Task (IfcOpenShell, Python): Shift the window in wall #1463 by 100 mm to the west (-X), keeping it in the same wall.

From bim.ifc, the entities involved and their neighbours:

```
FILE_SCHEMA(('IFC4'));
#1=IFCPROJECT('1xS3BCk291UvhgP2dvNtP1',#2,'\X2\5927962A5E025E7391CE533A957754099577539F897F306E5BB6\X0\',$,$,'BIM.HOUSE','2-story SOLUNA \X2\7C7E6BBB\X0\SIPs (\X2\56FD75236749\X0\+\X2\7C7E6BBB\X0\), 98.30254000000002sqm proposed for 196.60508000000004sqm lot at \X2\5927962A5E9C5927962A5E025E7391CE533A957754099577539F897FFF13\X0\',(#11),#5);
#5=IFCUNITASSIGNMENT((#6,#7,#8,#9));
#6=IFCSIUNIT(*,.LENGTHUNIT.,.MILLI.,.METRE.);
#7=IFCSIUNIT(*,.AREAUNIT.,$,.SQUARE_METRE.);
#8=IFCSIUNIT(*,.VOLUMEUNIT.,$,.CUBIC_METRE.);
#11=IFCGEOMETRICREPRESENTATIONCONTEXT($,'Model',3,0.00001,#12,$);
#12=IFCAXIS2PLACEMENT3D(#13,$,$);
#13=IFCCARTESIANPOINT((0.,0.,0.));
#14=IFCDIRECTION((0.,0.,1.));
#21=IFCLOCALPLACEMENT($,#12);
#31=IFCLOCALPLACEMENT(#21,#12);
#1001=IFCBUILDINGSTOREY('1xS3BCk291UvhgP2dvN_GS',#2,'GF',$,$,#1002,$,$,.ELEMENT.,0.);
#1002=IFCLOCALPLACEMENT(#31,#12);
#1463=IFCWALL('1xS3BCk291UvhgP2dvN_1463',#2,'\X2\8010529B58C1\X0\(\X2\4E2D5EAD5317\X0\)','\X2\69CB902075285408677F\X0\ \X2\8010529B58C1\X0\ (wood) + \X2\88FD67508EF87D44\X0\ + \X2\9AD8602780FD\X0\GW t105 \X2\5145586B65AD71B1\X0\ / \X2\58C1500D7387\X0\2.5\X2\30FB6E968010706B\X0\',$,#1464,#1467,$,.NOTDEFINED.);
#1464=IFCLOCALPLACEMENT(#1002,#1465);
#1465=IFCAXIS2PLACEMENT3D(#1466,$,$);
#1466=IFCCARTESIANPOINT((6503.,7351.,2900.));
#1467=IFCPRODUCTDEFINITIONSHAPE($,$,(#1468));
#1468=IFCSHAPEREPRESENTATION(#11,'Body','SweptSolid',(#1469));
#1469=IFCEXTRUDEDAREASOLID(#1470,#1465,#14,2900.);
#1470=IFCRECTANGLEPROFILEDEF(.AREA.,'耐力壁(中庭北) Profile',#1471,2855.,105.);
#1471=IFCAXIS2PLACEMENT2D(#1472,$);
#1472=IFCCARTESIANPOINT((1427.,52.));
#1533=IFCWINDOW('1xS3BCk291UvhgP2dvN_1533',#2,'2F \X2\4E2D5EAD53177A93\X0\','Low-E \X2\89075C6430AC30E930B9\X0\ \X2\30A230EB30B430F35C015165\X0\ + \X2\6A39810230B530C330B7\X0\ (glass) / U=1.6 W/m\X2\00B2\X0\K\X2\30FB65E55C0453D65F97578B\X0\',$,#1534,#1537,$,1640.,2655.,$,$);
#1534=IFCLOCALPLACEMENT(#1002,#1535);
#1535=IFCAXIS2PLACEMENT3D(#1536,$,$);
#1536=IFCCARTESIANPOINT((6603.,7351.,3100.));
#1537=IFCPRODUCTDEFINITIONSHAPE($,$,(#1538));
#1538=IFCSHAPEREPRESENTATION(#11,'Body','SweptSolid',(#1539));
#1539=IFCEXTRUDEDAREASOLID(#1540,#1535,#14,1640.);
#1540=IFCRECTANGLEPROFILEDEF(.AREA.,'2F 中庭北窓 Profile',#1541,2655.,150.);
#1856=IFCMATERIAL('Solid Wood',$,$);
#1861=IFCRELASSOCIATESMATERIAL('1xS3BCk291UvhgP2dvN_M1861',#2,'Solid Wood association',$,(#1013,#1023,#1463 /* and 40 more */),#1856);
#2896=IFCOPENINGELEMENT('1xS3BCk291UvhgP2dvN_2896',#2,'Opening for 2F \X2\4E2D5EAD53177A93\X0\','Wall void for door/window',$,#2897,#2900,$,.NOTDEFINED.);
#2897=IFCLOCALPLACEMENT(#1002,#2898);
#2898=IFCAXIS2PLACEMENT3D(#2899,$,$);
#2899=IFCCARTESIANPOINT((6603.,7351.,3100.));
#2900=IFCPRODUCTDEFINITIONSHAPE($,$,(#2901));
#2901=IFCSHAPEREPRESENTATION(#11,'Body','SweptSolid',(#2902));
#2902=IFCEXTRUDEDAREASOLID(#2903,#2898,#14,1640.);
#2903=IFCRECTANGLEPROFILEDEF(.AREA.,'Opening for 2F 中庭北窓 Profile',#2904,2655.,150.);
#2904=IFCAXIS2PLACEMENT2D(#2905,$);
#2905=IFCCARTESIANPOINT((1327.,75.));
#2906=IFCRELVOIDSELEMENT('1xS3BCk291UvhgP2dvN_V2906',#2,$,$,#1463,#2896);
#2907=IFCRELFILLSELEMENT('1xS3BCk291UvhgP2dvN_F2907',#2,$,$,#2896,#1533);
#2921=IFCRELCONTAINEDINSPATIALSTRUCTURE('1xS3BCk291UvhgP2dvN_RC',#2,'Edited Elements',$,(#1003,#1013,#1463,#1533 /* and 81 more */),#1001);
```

```python
import ifcopenshell
import ifcopenshell.api.geometry
import ifcopenshell.util.placement
import ifcopenshell.util.unit

model = ifcopenshell.open("bim.ifc")
unit_scale = ifcopenshell.util.unit.calculate_unit_scale(model)

window = model.by_id(1533)
opening = window.FillsVoids[0].RelatingOpeningElement
wall = opening.VoidsElements[0].RelatingBuildingElement

wall_matrix = ifcopenshell.util.placement.get_local_placement(wall.ObjectPlacement)
shift = wall_matrix[:3, 0] * -0.1 / unit_scale
before = ifcopenshell.util.placement.get_local_placement(window.ObjectPlacement)[:3, 3].copy()

# The window is not placed relative to its opening, so move both.
for product in (opening, window):
    matrix = ifcopenshell.util.placement.get_local_placement(product.ObjectPlacement)
    matrix[:3, 3] += shift
    ifcopenshell.api.geometry.edit_object_placement(model, product=product, matrix=matrix, is_si=False)

after = ifcopenshell.util.placement.get_local_placement(window.ObjectPlacement)[:3, 3]
print("window moved by", (after - before).round(3) + 0.0)

model.write("bim-out.ifc")
```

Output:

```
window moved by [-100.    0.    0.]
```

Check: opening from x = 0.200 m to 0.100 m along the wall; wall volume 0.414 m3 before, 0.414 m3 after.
